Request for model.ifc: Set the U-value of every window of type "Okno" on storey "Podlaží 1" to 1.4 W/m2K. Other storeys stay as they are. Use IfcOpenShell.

First a look at what the model holds.

```python
import ifcopenshell
import ifcopenshell.util.element

model = ifcopenshell.open("model.ifc")
print(model.schema)
storey = next(s for s in model.by_type("IfcBuildingStorey") if s.Name == "Podlaží 1")
windows = [e for e in ifcopenshell.util.element.get_decomposition(storey) if e.is_a("IfcWindow")]
seen = {}
for e in windows:
    element_type = ifcopenshell.util.element.get_type(e)
    key = (element_type.Name if element_type != e and element_type else None, ifcopenshell.util.element.get_pset(e, "Pset_WindowCommon", "ThermalTransmittance"))
    seen[key] = seen.get(key, 0) + 1
for (name, value), count in sorted(seen.items(), key=str):
    print(count, "x", name, "|", value)
```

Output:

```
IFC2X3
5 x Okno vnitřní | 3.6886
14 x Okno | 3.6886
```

```python
import ifcopenshell
import ifcopenshell.api.pset
import ifcopenshell.util.element

model = ifcopenshell.open("model.ifc")

storey = next(s for s in model.by_type("IfcBuildingStorey") if s.Name == "Podlaží 1")
windows = [e for e in ifcopenshell.util.element.get_decomposition(storey) if e.is_a("IfcWindow")]

count = 0
for e in windows:
    element_type = ifcopenshell.util.element.get_type(e)
    if element_type in (None, e) or element_type.Name != "Okno":
        continue
    # add_pset returns the element's existing set when there is one.
    pset = ifcopenshell.api.pset.add_pset(model, product=e, name="Pset_WindowCommon")
    ifcopenshell.api.pset.edit_pset(model, pset=pset, properties={"ThermalTransmittance": 1.4})
    count += 1

print(count, "windows updated")

model.write("model_updated.ifc")
```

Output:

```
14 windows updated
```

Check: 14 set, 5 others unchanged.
